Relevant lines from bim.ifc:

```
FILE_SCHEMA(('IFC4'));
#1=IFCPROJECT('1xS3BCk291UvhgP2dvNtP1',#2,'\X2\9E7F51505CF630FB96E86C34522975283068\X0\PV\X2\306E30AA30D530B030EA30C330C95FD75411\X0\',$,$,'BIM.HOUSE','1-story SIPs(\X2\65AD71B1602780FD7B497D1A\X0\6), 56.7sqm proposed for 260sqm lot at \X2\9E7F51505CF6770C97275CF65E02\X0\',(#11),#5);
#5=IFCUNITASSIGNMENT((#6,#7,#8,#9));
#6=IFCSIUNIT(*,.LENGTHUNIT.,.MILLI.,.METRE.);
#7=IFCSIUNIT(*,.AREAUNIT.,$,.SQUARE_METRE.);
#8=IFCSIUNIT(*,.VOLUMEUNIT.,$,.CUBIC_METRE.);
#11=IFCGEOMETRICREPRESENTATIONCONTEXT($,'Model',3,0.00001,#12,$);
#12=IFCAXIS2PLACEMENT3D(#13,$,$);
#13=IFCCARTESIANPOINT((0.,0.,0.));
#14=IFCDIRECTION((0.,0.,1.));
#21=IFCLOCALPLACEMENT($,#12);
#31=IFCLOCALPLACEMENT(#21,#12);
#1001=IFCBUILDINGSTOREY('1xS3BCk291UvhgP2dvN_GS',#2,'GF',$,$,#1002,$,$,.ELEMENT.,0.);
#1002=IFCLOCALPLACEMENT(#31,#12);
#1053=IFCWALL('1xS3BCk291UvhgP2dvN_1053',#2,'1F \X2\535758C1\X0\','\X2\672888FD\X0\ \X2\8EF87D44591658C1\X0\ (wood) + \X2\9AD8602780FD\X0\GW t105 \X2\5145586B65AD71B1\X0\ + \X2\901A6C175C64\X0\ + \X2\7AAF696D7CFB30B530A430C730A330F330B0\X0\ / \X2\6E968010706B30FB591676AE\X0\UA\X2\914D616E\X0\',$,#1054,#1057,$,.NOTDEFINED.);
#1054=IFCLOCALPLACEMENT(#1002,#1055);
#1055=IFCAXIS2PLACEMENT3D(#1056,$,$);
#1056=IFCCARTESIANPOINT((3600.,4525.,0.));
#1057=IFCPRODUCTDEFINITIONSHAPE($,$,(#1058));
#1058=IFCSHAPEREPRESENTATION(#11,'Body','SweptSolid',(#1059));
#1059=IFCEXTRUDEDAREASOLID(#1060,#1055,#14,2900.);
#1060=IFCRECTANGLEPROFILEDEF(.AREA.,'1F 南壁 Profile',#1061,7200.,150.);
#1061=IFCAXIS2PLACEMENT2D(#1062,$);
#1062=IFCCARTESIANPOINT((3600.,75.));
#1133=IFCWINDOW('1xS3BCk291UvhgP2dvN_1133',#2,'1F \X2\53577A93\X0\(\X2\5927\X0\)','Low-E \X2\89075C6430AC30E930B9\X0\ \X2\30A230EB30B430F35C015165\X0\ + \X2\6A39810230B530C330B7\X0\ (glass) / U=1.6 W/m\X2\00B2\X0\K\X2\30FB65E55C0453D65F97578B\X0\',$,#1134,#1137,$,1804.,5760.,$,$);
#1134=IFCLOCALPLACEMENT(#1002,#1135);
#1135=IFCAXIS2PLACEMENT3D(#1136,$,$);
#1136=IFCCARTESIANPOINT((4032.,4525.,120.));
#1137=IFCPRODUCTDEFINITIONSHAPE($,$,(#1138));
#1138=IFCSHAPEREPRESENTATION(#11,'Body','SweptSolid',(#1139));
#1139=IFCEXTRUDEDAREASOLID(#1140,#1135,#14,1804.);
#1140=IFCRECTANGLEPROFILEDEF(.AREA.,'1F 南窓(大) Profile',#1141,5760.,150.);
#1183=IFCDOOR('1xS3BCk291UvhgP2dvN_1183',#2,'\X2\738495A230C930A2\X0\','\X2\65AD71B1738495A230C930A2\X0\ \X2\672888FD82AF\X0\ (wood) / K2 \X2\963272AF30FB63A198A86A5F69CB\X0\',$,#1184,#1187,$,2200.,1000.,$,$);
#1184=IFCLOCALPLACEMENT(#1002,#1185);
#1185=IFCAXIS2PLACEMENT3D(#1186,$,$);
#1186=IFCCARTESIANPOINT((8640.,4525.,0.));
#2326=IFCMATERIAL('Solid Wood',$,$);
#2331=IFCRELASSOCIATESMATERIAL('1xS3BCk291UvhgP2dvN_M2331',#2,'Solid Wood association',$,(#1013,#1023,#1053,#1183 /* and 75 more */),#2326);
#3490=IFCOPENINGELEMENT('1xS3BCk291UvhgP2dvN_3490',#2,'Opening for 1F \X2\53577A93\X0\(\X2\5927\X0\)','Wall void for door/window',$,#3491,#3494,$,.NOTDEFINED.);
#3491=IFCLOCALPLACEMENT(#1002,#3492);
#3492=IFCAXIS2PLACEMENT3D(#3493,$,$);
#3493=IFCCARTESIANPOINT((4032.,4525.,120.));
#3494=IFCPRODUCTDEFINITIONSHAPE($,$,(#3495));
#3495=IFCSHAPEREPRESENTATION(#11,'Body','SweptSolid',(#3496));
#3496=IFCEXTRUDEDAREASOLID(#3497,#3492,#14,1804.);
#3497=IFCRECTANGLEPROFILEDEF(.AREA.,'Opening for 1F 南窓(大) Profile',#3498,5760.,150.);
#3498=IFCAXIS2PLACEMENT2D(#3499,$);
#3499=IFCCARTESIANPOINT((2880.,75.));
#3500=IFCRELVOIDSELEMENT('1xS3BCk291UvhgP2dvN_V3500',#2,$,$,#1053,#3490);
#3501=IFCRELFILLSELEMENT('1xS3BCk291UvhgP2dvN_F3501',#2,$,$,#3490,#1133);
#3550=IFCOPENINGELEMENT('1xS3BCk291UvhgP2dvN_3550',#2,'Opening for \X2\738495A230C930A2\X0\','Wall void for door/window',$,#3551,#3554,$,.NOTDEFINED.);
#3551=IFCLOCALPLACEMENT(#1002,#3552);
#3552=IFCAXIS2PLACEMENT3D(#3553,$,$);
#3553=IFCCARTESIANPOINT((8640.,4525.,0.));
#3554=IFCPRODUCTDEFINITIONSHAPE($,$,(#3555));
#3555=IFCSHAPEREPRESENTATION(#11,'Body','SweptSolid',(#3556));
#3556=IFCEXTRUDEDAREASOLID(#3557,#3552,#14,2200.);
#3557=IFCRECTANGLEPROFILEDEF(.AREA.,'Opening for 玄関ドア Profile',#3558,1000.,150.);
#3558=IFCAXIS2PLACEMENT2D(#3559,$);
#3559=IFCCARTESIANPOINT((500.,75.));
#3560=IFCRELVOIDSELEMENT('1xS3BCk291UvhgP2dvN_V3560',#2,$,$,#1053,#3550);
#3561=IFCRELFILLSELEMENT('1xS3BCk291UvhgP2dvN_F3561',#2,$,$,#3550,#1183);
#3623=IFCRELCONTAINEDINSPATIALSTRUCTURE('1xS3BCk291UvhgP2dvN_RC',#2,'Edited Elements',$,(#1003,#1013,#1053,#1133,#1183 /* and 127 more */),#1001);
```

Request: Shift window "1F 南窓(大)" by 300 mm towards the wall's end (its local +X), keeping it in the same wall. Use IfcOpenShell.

```python
import ifcopenshell
import ifcopenshell.api.geometry
import ifcopenshell.util.placement
import ifcopenshell.util.unit

model = ifcopenshell.open("bim.ifc")
unit_scale = ifcopenshell.util.unit.calculate_unit_scale(model)

window = model.by_guid("1xS3BCk291UvhgP2dvN_1133")
opening = window.FillsVoids[0].RelatingOpeningElement
wall = opening.VoidsElements[0].RelatingBuildingElement

wall_matrix = ifcopenshell.util.placement.get_local_placement(wall.ObjectPlacement)
shift = wall_matrix[:3, 0] * 0.3 / unit_scale
before = ifcopenshell.util.placement.get_local_placement(window.ObjectPlacement)[:3, 3].copy()

# The window is not placed relative to its opening, so move both.
for product in (opening, window):
    matrix = ifcopenshell.util.placement.get_local_placement(product.ObjectPlacement)
    matrix[:3, 3] += shift
    ifcopenshell.api.geometry.edit_object_placement(model, product=product, matrix=matrix, is_si=False)

after = ifcopenshell.util.placement.get_local_placement(window.ObjectPlacement)[:3, 3]
print("window moved by", (after - before).round(3) + 0.0)

model.write("bim_updated.ifc")
```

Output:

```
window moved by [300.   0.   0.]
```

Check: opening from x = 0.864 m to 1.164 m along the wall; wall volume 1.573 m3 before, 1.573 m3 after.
